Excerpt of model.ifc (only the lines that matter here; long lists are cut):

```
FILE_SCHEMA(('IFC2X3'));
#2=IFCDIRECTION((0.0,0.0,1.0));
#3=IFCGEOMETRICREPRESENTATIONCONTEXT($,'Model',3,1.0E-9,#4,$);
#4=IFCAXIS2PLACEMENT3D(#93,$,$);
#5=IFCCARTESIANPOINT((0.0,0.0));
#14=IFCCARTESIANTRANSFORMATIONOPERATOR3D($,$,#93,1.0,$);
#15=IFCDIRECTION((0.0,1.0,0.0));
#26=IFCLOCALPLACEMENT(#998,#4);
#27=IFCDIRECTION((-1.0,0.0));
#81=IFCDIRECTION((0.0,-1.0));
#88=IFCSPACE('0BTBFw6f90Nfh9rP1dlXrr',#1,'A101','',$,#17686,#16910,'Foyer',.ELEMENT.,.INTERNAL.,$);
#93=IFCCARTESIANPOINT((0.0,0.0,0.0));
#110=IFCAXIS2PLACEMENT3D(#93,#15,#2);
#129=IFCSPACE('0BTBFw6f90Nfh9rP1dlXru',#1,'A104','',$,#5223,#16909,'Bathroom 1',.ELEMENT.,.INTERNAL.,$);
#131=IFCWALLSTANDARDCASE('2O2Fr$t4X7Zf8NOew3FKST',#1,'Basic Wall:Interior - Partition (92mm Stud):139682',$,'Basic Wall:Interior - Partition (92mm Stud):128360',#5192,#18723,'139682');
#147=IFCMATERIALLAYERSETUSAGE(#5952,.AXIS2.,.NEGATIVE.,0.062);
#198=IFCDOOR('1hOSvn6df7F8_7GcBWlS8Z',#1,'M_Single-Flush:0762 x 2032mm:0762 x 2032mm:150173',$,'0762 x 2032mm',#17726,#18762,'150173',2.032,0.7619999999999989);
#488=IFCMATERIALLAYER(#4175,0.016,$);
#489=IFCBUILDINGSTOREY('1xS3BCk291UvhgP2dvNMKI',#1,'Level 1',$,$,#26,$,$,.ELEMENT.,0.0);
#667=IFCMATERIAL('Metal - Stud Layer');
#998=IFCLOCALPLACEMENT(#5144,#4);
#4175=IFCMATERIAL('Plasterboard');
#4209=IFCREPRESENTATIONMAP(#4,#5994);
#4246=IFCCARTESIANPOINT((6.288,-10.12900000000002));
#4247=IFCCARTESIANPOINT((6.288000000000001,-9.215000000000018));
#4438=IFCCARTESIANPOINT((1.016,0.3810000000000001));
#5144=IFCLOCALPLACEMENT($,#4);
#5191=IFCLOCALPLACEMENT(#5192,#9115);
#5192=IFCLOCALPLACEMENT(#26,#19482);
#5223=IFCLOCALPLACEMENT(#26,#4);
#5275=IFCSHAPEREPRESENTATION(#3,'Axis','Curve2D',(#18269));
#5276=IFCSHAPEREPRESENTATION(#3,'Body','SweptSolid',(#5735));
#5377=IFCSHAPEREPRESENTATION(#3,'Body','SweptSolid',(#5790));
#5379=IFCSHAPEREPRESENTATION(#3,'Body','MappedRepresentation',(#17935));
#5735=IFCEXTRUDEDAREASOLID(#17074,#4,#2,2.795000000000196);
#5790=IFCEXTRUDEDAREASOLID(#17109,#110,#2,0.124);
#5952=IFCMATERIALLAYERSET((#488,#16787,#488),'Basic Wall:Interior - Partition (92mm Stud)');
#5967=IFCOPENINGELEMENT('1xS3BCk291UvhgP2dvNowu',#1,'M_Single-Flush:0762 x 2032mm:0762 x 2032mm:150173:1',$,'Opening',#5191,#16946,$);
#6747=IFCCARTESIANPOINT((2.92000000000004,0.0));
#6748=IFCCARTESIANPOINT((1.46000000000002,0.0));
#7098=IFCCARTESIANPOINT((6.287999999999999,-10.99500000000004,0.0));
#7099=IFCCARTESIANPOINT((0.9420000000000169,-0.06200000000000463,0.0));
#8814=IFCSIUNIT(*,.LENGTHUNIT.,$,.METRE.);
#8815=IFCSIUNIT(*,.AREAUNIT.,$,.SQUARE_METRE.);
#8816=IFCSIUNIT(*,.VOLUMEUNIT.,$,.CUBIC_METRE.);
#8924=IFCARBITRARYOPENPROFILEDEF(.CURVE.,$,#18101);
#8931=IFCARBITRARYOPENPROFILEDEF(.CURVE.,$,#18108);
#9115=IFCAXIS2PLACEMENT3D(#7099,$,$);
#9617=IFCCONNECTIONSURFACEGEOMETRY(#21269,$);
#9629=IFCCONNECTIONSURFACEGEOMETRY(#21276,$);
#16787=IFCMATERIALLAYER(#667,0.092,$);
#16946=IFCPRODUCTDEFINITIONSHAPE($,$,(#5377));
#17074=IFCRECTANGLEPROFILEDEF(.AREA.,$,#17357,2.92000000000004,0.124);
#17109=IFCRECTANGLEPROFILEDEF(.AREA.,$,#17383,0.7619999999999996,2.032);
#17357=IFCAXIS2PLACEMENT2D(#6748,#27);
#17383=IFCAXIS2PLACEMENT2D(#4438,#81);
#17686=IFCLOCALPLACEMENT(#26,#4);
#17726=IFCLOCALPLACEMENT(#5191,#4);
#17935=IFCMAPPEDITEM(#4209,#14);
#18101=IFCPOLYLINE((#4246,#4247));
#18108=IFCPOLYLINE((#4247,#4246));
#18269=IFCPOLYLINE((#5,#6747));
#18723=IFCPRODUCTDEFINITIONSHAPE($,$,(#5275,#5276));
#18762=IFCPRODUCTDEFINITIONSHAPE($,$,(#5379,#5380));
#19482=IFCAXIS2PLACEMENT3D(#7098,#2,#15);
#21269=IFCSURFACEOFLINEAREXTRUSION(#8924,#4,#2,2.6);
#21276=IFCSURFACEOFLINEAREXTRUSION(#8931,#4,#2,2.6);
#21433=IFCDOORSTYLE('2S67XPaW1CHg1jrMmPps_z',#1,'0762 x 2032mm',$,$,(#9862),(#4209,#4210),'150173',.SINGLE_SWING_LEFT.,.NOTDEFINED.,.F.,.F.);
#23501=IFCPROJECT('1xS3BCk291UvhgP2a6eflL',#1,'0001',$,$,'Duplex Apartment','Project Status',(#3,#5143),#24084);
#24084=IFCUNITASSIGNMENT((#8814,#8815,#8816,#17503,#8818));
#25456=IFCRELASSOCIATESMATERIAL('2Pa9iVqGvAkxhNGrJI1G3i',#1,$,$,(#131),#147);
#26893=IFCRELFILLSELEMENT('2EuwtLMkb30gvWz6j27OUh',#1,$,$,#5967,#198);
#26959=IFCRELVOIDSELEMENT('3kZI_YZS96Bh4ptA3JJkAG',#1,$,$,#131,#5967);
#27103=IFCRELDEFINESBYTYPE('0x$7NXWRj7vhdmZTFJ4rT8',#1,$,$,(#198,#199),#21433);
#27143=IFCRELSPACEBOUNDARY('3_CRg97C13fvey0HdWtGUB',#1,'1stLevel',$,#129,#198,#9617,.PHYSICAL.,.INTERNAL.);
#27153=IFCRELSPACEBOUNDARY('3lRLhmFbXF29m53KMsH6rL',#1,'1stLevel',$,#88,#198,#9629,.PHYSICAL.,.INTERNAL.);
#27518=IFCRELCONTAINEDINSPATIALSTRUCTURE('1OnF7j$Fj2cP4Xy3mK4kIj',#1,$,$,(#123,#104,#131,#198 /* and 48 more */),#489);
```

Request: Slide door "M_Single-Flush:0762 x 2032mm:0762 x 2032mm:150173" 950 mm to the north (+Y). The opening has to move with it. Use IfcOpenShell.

```python
import numpy as np
import ifcopenshell
import ifcopenshell.api.geometry
import ifcopenshell.util.placement

model = ifcopenshell.open("model.ifc")

door = model.by_id(198)
opening = door.FillsVoids[0].RelatingOpeningElement
wall = opening.VoidsElements[0].RelatingBuildingElement

wall_matrix = ifcopenshell.util.placement.get_local_placement(wall.ObjectPlacement)
shift = wall_matrix[:3, 0] * 0.95
before = ifcopenshell.util.placement.get_local_placement(door.ObjectPlacement)[:3, 3].copy()

# The door is placed relative to its opening, so it follows when the opening moves.
matrix = ifcopenshell.util.placement.get_local_placement(opening.ObjectPlacement)
matrix[:3, 3] += shift
ifcopenshell.api.geometry.edit_object_placement(
    model, product=opening, matrix=matrix, is_si=False, should_transform_children=True
)

# Space boundary surfaces are stored in each space's coordinates; move them too.
for rel in door.ProvidesBoundaries:
    if not rel.ConnectionGeometry:
        continue
    surface = rel.ConnectionGeometry.SurfaceOnRelatingElement
    space_matrix = ifcopenshell.util.placement.get_local_placement(rel.RelatingSpace.ObjectPlacement)
    point = np.array(surface.Position.Location.Coordinates) + space_matrix[:3, :3].T @ shift
    surface.Position = model.createIfcAxis2Placement3D(
        model.createIfcCartesianPoint(point.tolist()), surface.Position.Axis, surface.Position.RefDirection
    )

after = ifcopenshell.util.placement.get_local_placement(door.ObjectPlacement)[:3, 3]
print("door moved by", (after - before).round(3) + 0.0)

model.write("model-out.ifc")
```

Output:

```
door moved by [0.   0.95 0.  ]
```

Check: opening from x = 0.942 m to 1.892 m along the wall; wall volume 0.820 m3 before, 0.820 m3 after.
